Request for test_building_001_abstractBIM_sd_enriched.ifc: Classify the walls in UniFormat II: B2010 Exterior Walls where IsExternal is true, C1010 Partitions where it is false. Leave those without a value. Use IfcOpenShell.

First a look at what the model holds.

```python
import ifcopenshell
import ifcopenshell.util.element

model = ifcopenshell.open("test_building_001_abstractBIM_sd_enriched.ifc")
print(model.schema)
print("classifications:", [c.Name for c in model.by_type("IfcClassification")])
values = [ifcopenshell.util.element.get_pset(e, "Pset_WallCommon", "IsExternal") for e in model.by_type("IfcWall")]
for value in (True, False, None):
    print("IsExternal", value, values.count(value))
```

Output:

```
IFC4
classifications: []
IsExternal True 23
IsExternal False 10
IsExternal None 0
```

```python
import ifcopenshell
import ifcopenshell.api.classification
import ifcopenshell.util.element

model = ifcopenshell.open("test_building_001_abstractBIM_sd_enriched.ifc")

system = ifcopenshell.api.classification.add_classification(model, classification="UniFormat II")

walls = model.by_type("IfcWall")
external = {e: ifcopenshell.util.element.get_pset(e, "Pset_WallCommon", "IsExternal") for e in walls}
for flag, code, name in ((True, "B2010", "Exterior Walls"), (False, "C1010", "Partitions")):
    products = [e for e in walls if external[e] is flag]
    ifcopenshell.api.classification.add_reference(
        model, products=products, classification=system, identification=code, name=name
    )
    print(code, len(products))

model.write("test_building_001_abstractBIM_sd_enriched_rev.ifc")
```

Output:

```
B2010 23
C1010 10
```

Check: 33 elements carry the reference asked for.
